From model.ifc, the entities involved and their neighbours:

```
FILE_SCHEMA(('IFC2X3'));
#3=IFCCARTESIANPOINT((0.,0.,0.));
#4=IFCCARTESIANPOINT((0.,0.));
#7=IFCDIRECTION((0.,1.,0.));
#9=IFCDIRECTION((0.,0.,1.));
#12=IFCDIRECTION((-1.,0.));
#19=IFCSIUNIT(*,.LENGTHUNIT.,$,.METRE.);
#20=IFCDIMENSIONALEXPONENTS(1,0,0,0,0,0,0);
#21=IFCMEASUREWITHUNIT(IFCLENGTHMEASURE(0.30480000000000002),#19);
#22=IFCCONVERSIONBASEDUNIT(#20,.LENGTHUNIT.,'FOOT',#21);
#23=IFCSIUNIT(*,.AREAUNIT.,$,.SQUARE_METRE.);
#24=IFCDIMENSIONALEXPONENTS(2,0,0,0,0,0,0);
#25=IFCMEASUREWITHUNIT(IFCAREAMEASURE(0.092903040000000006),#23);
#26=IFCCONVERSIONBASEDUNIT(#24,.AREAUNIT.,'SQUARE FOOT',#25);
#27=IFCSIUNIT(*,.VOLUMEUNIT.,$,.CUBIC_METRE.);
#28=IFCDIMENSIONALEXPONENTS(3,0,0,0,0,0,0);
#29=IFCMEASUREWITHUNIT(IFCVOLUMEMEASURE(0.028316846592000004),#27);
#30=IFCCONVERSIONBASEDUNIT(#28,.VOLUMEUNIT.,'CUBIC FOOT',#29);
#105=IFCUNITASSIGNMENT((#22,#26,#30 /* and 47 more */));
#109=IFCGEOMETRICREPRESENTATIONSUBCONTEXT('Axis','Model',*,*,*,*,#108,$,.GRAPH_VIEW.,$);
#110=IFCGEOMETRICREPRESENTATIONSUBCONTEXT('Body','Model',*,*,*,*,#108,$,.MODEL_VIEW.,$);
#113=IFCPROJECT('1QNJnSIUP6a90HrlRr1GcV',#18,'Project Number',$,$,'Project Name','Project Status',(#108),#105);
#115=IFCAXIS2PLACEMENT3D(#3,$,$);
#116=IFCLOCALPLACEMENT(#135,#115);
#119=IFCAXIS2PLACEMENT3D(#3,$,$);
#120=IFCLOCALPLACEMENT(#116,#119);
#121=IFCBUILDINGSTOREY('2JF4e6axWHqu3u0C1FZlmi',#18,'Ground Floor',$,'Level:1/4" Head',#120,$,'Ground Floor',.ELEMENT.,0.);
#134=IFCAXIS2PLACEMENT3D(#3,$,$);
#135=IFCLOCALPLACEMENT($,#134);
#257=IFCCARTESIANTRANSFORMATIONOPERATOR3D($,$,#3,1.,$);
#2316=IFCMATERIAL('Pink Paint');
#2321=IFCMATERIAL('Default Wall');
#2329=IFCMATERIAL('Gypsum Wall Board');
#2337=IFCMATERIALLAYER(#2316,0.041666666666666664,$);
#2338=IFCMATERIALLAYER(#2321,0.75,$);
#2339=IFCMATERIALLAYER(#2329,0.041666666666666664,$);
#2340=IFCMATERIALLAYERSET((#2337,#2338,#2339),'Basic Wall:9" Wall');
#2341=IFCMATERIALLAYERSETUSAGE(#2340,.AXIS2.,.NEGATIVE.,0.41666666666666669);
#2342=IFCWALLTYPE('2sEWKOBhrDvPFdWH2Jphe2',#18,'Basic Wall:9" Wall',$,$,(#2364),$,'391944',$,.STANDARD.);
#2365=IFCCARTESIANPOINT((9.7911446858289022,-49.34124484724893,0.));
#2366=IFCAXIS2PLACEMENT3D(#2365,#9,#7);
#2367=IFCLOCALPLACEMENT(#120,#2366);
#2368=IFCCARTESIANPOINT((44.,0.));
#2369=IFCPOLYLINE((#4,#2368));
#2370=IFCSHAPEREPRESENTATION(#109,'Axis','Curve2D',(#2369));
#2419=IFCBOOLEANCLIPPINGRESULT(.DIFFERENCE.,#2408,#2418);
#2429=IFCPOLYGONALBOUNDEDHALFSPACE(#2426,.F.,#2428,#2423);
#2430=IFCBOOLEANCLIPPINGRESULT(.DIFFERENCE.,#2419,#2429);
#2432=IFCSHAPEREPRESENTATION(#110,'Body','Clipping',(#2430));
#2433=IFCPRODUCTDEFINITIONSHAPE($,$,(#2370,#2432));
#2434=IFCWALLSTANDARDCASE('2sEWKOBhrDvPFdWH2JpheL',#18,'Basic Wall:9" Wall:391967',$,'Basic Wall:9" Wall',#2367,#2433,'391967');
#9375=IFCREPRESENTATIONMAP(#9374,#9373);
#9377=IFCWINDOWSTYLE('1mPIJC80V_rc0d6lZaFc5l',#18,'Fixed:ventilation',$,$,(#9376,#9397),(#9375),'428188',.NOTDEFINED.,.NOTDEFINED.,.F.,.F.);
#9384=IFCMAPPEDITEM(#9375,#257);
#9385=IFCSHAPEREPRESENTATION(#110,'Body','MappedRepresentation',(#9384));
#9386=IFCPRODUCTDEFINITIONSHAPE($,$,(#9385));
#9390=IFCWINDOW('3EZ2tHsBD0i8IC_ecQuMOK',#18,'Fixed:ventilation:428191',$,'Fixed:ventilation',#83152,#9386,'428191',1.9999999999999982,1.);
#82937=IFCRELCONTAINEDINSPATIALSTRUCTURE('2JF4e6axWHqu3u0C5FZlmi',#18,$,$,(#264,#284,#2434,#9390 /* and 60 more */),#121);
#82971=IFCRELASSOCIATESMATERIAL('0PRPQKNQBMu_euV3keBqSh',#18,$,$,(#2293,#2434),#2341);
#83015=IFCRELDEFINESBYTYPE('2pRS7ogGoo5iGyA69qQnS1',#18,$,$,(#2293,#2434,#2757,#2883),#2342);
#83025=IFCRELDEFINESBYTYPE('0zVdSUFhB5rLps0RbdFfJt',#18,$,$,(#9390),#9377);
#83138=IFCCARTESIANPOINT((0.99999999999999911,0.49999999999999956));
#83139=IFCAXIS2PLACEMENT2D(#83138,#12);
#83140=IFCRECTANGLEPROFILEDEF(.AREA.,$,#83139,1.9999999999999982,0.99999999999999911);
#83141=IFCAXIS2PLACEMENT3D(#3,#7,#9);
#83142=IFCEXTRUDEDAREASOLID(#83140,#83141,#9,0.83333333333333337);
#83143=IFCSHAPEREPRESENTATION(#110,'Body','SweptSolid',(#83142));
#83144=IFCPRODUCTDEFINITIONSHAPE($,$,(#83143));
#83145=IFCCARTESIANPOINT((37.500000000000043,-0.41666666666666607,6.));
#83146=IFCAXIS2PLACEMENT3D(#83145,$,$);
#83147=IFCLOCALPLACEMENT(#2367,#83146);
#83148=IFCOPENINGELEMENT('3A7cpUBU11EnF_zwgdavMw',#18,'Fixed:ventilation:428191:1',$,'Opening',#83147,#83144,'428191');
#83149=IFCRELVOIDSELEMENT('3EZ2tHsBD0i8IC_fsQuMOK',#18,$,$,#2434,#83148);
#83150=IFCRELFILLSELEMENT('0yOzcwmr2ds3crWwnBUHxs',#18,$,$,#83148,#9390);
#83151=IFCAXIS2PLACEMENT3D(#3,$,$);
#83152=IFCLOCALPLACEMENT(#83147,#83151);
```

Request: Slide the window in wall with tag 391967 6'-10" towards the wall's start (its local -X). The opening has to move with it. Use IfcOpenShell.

```python
import ifcopenshell
import ifcopenshell.api.geometry
import ifcopenshell.util.placement
import ifcopenshell.util.unit

model = ifcopenshell.open("model.ifc")
unit_scale = ifcopenshell.util.unit.calculate_unit_scale(model)

window = model.by_guid("3EZ2tHsBD0i8IC_ecQuMOK")
opening = window.FillsVoids[0].RelatingOpeningElement
wall = opening.VoidsElements[0].RelatingBuildingElement

wall_matrix = ifcopenshell.util.placement.get_local_placement(wall.ObjectPlacement)
shift = wall_matrix[:3, 0] * -82 * 0.0254 / unit_scale
before = ifcopenshell.util.placement.get_local_placement(window.ObjectPlacement)[:3, 3].copy()

# The window is placed relative to its opening, so it follows when the opening moves.
matrix = ifcopenshell.util.placement.get_local_placement(opening.ObjectPlacement)
matrix[:3, 3] += shift
ifcopenshell.api.geometry.edit_object_placement(
    model, product=opening, matrix=matrix, is_si=False, should_transform_children=True
)

after = ifcopenshell.util.placement.get_local_placement(window.ObjectPlacement)[:3, 3]
print("window moved by", (after - before).round(3) + 0.0)

model.write("model_rev.ifc")
```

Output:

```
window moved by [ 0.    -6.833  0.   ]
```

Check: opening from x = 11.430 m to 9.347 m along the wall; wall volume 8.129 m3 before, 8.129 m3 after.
